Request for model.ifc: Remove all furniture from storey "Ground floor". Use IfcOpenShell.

First a look at what the model holds.

```python
import ifcopenshell
import ifcopenshell.util.element

model = ifcopenshell.open("model.ifc")
print(model.schema)
storey = next(s for s in model.by_type("IfcBuildingStorey") if s.Name == "Ground floor")
furniture = [e for e in ifcopenshell.util.element.get_decomposition(storey) if e.is_a("IfcFurnishingElement")]
seen = {}
for e in furniture:
    element_type = ifcopenshell.util.element.get_type(e)
    name = element_type.Name if element_type not in (None, e) else None
    seen[name] = seen.get(name, 0) + 1
for name, count in sorted(seen.items(), key=str):
    print(count, "x", name)
```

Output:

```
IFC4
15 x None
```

```python
import ifcopenshell
import ifcopenshell.api.root
import ifcopenshell.util.element

model = ifcopenshell.open("model.ifc")

storey = next(s for s in model.by_type("IfcBuildingStorey") if s.Name == "Ground floor")
furniture = [e for e in ifcopenshell.util.element.get_decomposition(storey) if e.is_a("IfcFurnishingElement")]

for e in furniture:
    ifcopenshell.api.root.remove_product(model, product=e)
print(len(furniture), "removed")

model.write("model_updated.ifc")
```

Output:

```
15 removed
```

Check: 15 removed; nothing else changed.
